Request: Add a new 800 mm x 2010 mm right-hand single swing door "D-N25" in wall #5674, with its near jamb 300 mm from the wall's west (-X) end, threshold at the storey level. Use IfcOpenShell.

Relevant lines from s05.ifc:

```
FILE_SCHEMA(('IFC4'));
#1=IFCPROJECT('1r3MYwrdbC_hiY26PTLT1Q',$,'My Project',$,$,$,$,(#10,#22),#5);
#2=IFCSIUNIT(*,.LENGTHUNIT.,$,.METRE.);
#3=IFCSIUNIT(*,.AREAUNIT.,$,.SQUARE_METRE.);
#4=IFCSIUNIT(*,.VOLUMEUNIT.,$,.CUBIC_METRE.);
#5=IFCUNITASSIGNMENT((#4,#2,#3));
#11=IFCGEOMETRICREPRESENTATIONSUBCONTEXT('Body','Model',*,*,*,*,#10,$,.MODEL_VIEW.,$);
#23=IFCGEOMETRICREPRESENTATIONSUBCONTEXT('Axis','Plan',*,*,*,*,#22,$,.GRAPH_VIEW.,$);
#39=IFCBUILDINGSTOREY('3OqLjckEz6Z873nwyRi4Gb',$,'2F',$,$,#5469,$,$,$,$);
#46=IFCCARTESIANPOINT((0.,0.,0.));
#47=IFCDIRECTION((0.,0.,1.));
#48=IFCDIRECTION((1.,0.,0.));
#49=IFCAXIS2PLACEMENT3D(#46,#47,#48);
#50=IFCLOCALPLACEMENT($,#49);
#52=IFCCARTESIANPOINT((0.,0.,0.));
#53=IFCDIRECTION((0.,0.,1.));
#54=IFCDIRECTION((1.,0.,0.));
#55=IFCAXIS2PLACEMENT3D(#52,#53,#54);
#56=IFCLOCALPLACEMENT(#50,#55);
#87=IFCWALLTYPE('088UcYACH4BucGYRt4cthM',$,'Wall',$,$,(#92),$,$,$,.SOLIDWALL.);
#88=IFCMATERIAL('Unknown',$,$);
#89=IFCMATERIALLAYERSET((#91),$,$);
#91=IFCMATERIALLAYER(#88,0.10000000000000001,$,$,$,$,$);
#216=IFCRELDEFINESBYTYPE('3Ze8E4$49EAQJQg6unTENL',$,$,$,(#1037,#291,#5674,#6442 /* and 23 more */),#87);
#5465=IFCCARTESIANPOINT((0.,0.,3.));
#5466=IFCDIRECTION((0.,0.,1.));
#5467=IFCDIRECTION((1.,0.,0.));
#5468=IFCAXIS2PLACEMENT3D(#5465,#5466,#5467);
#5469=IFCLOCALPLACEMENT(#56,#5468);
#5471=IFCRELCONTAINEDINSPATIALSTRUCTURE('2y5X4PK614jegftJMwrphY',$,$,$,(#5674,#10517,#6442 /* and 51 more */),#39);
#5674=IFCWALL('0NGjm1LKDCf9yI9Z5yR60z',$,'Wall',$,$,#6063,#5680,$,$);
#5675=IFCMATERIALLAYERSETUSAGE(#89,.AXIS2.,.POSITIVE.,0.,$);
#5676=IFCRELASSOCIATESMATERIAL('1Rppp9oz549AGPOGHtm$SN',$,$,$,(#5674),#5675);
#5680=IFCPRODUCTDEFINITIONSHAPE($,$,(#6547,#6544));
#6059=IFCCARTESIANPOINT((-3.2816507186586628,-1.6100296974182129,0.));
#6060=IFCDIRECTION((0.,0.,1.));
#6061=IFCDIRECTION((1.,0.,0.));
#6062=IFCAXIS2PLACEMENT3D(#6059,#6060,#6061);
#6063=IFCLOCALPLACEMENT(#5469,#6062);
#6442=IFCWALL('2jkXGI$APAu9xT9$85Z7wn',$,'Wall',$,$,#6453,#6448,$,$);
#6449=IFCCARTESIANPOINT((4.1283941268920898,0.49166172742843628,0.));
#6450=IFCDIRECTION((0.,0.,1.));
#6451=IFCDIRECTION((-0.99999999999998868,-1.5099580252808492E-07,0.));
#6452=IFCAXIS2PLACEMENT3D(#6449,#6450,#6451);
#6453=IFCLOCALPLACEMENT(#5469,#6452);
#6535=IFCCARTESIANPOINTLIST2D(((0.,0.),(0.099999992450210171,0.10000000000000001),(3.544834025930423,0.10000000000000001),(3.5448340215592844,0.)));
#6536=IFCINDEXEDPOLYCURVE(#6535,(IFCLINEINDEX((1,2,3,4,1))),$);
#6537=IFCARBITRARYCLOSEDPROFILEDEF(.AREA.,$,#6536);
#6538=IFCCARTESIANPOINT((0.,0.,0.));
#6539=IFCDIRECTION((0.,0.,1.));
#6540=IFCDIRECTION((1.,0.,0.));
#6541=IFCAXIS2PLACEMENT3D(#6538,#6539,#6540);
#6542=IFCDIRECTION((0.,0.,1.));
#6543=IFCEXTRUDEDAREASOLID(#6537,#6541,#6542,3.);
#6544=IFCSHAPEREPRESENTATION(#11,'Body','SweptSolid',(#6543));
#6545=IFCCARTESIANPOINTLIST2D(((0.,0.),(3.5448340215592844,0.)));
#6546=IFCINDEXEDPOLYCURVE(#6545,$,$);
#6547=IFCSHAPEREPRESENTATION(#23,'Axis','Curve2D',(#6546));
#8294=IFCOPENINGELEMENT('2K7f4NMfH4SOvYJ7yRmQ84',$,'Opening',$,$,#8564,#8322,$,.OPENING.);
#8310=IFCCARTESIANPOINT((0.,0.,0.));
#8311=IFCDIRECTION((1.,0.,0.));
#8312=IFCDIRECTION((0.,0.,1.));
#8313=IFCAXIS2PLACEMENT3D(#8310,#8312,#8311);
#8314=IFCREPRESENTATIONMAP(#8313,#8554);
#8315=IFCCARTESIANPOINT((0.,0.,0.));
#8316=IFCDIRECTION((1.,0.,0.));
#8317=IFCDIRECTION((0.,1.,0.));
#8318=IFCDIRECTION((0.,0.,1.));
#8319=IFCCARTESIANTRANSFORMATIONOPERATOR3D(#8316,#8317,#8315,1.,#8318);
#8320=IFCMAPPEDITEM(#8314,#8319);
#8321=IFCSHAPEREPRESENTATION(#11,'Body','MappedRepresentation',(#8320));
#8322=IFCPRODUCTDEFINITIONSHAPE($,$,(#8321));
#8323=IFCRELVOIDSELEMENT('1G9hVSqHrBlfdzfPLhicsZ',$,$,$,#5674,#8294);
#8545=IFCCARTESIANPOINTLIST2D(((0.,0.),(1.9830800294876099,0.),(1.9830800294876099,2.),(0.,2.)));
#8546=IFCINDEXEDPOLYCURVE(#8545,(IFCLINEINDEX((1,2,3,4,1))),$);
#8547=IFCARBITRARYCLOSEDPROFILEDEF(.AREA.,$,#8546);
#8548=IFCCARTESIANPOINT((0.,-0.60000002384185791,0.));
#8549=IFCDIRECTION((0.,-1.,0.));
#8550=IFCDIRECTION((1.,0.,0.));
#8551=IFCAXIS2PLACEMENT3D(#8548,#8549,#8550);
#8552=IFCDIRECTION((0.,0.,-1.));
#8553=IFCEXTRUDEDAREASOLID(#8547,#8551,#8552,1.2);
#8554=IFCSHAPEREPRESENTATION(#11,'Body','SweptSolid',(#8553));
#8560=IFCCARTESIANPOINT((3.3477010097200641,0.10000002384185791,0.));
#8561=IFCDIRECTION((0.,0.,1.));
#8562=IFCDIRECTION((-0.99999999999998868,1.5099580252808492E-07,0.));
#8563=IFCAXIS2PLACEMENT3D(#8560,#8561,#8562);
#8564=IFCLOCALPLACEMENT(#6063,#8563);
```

```python
import numpy as np
import ifcopenshell
import ifcopenshell.api.feature
import ifcopenshell.api.geometry
import ifcopenshell.api.root
import ifcopenshell.api.spatial
import ifcopenshell.geom
import ifcopenshell.util.element
import ifcopenshell.util.placement
import ifcopenshell.util.representation
import ifcopenshell.util.shape
import ifcopenshell.util.unit

model = ifcopenshell.open("s05.ifc")
unit_scale = ifcopenshell.util.unit.calculate_unit_scale(model)
settings = ifcopenshell.geom.settings()


def volume(element):
    """Net volume in cubic metres, openings subtracted."""
    shape = ifcopenshell.geom.create_shape(settings, element)
    return ifcopenshell.util.shape.get_volume(shape.geometry)


wall = model.by_guid("0NGjm1LKDCf9yI9Z5yR60z")
storey = ifcopenshell.util.element.get_container(wall, ifc_class="IfcBuildingStorey")
context = ifcopenshell.util.representation.get_context(model, "Model", "Body", "MODEL_VIEW")
before = volume(wall)

width, height, from_end, sill = 0.8, 2.01, 0.3, 0.0  # metres

# The wall runs along its own X axis, and the end named is its -X end.
wall_shape = ifcopenshell.geom.create_shape(settings, wall)
x, y, z = ifcopenshell.util.shape.get_vertices(wall_shape.geometry).T
start = x.min() + from_end
face, thickness = float(y.min()), float(y.max() - y.min())
wall_matrix = ifcopenshell.util.placement.get_local_placement(wall.ObjectPlacement)
level = ifcopenshell.util.placement.get_local_placement(storey.ObjectPlacement)[2, 3]


def in_wall(x, y):
    """Placement at x, y metres in the wall's axes, at sill height."""
    matrix = wall_matrix.copy()
    matrix[:, 3] = wall_matrix @ np.array([x / unit_scale, y / unit_scale, 0.0, 1.0])
    matrix[2, 3] = level + sill / unit_scale
    return matrix


# Opening: a box that overshoots both wall faces by 50 mm.
opening = ifcopenshell.api.root.create_entity(model, ifc_class="IfcOpeningElement", predefined_type="OPENING")
box = ifcopenshell.api.geometry.add_wall_representation(
    model, context=context, length=width, height=height, thickness=thickness + 0.1
)
ifcopenshell.api.geometry.assign_representation(model, product=opening, representation=box)
ifcopenshell.api.geometry.edit_object_placement(model, product=opening, matrix=in_wall(start, face - 0.05), is_si=False)
ifcopenshell.api.feature.add_feature(model, feature=opening, element=wall)

door = ifcopenshell.api.root.create_entity(model, ifc_class="IfcDoor", name="D-N25", predefined_type="DOOR")
door.OverallWidth, door.OverallHeight = width / unit_scale, height / unit_scale
door.OperationType = "SINGLE_SWING_RIGHT"
body = ifcopenshell.api.geometry.add_door_representation(
    model,
    context=context,
    overall_width=door.OverallWidth,
    overall_height=door.OverallHeight,
    operation_type="SINGLE_SWING_RIGHT",
    lining_properties={"LiningDepth": thickness / unit_scale, "ThresholdDepth": thickness / unit_scale},
)
ifcopenshell.api.geometry.assign_representation(model, product=door, representation=body)
ifcopenshell.api.spatial.assign_container(model, products=[door], relating_structure=storey)
ifcopenshell.api.feature.add_filling(model, opening=opening, element=door)

# The lining spans the wall, so the door starts at the wall face.
ifcopenshell.api.geometry.edit_object_placement(model, product=door, matrix=in_wall(start, face), is_si=False)

after = volume(wall)

print(f"wall volume {before:.3f} -> {after:.3f} m3")

model.write("s05_v2.ifc")
```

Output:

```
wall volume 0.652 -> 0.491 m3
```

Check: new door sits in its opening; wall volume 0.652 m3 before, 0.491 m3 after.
